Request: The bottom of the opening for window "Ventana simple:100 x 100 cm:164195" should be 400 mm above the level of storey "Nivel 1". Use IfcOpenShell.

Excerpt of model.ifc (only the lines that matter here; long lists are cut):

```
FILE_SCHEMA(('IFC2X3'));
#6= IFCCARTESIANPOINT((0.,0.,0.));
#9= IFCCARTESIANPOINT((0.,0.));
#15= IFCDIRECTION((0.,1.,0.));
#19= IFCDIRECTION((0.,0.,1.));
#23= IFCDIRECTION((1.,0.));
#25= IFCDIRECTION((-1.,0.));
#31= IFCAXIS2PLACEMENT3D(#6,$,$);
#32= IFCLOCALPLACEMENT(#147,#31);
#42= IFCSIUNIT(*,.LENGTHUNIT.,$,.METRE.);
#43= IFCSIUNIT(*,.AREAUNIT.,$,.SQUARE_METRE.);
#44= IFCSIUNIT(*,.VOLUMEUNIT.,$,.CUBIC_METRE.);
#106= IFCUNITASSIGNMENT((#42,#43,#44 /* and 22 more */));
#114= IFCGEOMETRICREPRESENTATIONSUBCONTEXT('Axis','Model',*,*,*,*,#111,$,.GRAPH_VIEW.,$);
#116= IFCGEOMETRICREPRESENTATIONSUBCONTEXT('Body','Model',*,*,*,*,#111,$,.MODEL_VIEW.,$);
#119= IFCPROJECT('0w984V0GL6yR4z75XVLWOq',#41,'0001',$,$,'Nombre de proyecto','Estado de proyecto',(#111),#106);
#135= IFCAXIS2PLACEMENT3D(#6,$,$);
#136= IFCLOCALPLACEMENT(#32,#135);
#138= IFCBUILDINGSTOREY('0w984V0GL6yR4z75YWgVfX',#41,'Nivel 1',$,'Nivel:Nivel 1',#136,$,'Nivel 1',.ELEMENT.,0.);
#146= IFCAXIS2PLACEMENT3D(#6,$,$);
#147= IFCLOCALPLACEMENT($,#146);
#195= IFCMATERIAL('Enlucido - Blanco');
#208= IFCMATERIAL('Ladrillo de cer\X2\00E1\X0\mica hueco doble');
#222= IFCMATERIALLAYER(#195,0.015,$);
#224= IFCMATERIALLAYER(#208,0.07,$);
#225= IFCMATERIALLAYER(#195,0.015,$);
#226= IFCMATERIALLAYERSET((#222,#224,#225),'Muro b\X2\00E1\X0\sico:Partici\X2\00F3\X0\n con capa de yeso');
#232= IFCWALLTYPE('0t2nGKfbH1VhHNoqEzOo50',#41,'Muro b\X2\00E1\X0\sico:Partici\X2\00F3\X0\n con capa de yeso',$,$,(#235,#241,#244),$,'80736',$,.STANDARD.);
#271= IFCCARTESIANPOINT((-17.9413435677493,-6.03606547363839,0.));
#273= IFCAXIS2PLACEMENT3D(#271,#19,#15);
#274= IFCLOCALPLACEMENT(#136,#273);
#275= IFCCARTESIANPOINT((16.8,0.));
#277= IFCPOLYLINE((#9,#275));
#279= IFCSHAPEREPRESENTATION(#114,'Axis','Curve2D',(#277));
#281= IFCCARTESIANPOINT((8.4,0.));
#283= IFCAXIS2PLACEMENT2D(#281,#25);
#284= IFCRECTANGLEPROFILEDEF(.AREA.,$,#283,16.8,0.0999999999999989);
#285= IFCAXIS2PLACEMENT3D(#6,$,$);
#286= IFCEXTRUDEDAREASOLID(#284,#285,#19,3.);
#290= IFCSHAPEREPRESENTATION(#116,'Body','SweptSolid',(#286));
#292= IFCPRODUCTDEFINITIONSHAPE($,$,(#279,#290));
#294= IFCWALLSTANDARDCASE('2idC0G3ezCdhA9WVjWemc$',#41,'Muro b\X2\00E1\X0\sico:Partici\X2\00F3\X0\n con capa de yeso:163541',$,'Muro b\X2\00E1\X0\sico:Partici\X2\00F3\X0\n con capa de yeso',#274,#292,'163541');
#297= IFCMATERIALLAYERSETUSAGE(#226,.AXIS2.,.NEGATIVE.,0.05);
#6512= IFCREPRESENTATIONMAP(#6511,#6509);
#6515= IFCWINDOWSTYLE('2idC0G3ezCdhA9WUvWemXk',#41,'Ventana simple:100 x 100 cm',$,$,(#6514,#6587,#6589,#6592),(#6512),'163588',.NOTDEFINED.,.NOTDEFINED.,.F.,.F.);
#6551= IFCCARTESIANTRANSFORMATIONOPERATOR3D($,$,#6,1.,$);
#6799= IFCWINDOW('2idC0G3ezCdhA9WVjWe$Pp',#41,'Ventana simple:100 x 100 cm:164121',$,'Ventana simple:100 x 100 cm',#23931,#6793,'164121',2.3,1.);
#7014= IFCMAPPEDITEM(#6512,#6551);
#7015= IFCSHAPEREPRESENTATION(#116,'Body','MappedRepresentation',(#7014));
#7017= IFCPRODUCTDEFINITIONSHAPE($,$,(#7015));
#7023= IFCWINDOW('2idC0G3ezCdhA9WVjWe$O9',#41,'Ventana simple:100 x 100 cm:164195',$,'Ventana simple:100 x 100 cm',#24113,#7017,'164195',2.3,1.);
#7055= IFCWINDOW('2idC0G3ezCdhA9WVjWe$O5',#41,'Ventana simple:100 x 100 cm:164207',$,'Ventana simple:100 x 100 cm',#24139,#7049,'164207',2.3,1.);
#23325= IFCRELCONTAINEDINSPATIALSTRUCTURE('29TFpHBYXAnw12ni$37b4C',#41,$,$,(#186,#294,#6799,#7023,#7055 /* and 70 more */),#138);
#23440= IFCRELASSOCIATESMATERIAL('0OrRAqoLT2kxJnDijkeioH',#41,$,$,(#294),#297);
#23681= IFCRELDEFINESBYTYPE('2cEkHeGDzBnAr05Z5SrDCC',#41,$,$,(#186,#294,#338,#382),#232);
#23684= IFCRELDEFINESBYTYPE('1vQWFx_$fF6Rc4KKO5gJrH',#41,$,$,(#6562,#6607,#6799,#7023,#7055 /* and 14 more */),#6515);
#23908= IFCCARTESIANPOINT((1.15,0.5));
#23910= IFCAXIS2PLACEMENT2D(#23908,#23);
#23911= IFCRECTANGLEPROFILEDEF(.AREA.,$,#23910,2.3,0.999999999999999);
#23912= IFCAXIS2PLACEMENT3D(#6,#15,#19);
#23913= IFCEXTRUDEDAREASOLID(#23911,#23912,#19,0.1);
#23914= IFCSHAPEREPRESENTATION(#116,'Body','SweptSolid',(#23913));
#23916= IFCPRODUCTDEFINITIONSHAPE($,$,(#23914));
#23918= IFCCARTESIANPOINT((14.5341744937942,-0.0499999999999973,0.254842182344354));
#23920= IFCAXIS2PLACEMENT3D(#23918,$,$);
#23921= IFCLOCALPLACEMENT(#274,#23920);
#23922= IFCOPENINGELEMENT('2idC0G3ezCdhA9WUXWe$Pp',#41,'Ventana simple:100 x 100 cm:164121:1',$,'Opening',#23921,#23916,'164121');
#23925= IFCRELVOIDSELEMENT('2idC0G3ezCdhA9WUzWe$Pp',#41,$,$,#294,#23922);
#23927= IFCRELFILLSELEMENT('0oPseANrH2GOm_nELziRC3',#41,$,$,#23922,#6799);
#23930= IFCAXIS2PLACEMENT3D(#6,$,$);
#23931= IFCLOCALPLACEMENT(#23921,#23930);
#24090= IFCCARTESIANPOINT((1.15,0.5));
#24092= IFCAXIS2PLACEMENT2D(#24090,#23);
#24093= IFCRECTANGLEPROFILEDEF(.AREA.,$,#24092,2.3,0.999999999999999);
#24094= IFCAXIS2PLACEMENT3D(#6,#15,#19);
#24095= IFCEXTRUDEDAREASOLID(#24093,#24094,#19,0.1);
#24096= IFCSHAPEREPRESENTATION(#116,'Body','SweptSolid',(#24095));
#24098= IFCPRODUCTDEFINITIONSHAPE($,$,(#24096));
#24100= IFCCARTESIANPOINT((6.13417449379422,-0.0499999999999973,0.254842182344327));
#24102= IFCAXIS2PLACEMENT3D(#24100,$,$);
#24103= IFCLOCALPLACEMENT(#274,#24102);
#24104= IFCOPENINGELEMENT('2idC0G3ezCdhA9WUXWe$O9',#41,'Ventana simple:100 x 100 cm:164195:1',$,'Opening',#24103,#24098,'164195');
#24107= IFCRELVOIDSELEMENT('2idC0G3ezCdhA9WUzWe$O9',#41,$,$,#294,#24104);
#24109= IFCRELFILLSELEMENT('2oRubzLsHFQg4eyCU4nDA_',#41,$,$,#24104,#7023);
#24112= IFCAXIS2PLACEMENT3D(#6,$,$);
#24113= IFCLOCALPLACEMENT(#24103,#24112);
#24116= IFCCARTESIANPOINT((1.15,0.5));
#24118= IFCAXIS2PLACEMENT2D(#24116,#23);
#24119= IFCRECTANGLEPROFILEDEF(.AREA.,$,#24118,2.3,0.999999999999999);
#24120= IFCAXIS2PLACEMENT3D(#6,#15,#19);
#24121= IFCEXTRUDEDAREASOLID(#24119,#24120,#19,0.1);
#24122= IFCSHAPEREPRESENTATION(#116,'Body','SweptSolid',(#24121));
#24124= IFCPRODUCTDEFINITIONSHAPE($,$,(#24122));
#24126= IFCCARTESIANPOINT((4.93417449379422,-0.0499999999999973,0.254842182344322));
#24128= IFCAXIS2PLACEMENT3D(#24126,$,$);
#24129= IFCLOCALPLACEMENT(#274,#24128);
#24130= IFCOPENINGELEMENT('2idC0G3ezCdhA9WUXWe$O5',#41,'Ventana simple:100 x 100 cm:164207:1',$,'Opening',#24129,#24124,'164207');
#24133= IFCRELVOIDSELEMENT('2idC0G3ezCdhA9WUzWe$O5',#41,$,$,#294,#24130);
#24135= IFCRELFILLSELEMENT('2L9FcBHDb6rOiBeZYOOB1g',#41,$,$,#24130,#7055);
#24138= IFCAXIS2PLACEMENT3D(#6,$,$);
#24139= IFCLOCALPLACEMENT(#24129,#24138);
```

```python
import numpy as np
import ifcopenshell
import ifcopenshell.api.geometry
import ifcopenshell.geom
import ifcopenshell.util.element
import ifcopenshell.util.placement
import ifcopenshell.util.shape
import ifcopenshell.util.unit

model = ifcopenshell.open("model.ifc")
unit_scale = ifcopenshell.util.unit.calculate_unit_scale(model)

window = model.by_guid("2idC0G3ezCdhA9WVjWe$O9")
opening = window.FillsVoids[0].RelatingOpeningElement
storey = ifcopenshell.util.element.get_container(window, ifc_class="IfcBuildingStorey")
level = ifcopenshell.util.placement.get_local_placement(storey.ObjectPlacement)[2, 3]

# The opening's origin need not be at the sill, so measure its lowest point.
shape = ifcopenshell.geom.create_shape(ifcopenshell.geom.settings(), opening)
bottom = ifcopenshell.util.shape.get_shape_bottom_elevation(shape, shape.geometry) / unit_scale
dz = level + 0.4 / unit_scale - bottom

shift = np.array([0.0, 0.0, dz])
# The window is placed relative to its opening, so it follows when the opening moves.
matrix = ifcopenshell.util.placement.get_local_placement(opening.ObjectPlacement)
matrix[:3, 3] += shift
ifcopenshell.api.geometry.edit_object_placement(
    model, product=opening, matrix=matrix, is_si=False, should_transform_children=True
)

print(f"moved by {dz * unit_scale:+.3f} m")

model.write("model_edited.ifc")
```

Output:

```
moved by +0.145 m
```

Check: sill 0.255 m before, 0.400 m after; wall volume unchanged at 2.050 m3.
